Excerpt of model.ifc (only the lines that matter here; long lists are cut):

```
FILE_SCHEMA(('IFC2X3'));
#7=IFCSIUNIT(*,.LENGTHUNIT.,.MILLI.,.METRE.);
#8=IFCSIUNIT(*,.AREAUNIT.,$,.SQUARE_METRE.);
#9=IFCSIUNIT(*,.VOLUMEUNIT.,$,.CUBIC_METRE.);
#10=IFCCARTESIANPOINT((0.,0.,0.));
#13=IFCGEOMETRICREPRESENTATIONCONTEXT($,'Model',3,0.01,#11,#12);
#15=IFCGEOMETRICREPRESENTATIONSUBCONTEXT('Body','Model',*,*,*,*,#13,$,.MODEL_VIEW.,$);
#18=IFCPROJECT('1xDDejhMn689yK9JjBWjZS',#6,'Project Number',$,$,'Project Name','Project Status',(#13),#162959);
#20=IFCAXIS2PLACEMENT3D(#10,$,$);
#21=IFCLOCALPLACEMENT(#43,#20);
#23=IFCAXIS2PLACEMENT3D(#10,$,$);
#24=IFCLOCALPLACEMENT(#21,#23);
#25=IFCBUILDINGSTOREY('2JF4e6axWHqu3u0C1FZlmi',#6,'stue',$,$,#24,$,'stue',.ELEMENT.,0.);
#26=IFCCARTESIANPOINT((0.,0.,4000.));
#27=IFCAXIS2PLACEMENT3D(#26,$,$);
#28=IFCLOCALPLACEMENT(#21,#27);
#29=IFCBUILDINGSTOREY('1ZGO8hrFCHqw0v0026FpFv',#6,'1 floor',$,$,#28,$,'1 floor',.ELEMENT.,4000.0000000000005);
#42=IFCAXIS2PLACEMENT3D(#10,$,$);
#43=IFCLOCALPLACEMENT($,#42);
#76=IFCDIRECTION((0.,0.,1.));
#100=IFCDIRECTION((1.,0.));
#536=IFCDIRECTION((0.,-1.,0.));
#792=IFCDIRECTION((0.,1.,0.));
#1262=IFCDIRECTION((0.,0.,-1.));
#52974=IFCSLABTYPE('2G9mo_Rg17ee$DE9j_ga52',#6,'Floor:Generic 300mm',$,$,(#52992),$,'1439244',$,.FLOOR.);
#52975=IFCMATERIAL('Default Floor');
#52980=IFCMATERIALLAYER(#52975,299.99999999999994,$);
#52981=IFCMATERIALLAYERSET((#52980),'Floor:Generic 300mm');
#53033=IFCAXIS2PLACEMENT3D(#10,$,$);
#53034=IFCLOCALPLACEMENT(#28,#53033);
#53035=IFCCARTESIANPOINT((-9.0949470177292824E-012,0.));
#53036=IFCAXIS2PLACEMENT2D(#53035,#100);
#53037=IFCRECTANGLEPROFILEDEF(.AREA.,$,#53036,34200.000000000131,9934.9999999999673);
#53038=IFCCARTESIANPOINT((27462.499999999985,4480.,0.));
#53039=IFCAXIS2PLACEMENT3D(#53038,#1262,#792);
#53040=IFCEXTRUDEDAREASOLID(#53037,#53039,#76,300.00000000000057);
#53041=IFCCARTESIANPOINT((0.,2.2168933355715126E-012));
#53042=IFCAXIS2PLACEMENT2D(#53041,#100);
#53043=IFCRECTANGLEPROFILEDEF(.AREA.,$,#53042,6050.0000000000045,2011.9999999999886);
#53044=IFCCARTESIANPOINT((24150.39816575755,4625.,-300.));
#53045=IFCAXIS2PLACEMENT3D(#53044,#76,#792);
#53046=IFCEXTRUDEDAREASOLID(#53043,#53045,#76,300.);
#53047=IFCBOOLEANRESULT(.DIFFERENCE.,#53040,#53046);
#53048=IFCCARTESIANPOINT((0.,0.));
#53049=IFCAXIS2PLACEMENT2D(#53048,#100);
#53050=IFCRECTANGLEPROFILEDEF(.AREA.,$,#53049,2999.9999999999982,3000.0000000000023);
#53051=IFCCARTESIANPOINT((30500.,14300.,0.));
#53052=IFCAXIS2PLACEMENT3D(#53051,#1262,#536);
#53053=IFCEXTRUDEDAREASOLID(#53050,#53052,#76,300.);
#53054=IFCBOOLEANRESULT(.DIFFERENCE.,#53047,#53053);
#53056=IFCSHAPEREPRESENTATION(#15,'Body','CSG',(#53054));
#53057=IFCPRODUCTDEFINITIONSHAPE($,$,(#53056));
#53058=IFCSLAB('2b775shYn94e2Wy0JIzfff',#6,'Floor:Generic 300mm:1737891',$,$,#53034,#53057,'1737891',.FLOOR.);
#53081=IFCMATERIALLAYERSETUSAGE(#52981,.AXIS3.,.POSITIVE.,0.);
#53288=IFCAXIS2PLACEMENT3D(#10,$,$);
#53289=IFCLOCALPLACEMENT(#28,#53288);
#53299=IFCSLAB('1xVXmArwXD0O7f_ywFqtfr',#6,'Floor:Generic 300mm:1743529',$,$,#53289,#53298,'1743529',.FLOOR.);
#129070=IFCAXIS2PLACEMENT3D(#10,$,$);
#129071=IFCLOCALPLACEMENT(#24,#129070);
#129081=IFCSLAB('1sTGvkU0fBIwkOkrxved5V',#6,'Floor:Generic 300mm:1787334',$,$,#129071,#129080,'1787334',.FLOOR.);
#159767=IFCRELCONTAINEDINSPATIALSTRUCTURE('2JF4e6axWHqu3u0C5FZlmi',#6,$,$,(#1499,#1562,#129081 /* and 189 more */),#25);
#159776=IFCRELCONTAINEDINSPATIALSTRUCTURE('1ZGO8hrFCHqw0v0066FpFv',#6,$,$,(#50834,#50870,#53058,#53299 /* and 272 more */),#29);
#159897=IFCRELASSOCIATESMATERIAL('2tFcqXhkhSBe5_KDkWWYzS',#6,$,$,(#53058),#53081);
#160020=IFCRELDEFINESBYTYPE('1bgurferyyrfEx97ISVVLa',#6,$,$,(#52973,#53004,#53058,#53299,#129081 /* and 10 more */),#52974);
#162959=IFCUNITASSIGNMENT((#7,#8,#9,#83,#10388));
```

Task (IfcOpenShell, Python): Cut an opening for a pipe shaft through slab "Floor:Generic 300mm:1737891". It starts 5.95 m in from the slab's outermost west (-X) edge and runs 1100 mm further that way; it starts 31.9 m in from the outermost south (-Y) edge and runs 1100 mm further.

```python
import numpy as np
import ifcopenshell
import ifcopenshell.api.feature
import ifcopenshell.api.geometry
import ifcopenshell.api.root
import ifcopenshell.geom
import ifcopenshell.util.placement
import ifcopenshell.util.representation
import ifcopenshell.util.shape
import ifcopenshell.util.unit

model = ifcopenshell.open("model.ifc")
unit_scale = ifcopenshell.util.unit.calculate_unit_scale(model)
settings = ifcopenshell.geom.settings()


def volume(element):
    """Net volume in cubic metres, openings subtracted."""
    shape = ifcopenshell.geom.create_shape(settings, element)
    return ifcopenshell.util.shape.get_volume(shape.geometry)


slab = model.by_guid("2b775shYn94e2Wy0JIzfff")
before = volume(slab)

# Extent in the slab's own axes, in metres. The edges named are its -X and -Y sides.
slab_shape = ifcopenshell.geom.create_shape(settings, slab)
vertices = ifcopenshell.util.shape.get_vertices(slab_shape.geometry)
x_min, y_min, bottom = vertices.min(axis=0)
top = vertices[:, 2].max()

opening = ifcopenshell.api.root.create_entity(model, ifc_class="IfcOpeningElement", name="Pipe shaft opening")
context = ifcopenshell.util.representation.get_context(model, "Model", "Body", "MODEL_VIEW")
width, depth = 1.1, 1.1
outline = [(0.0, 0.0), (width, 0.0), (width, depth), (0.0, depth), (0.0, 0.0)]
# Overshoot both faces by 50 mm so the cut is clean.
shape = ifcopenshell.api.geometry.add_slab_representation(
    model, context=context, depth=top - bottom + 0.1, polyline=outline
)
ifcopenshell.api.geometry.assign_representation(model, product=opening, representation=shape)

matrix = ifcopenshell.util.placement.get_local_placement(slab.ObjectPlacement)
matrix[:, 3] = matrix @ np.append(np.array([x_min + 5.95, y_min + 31.9, bottom - 0.05]) / unit_scale, 1.0)
ifcopenshell.api.geometry.edit_object_placement(model, product=opening, matrix=matrix, is_si=False)
ifcopenshell.api.feature.add_feature(model, feature=opening, element=slab)

after = volume(slab)

print(f"slab volume {before:.3f} -> {after:.3f} m3")

model.write("model-out.ifc")
```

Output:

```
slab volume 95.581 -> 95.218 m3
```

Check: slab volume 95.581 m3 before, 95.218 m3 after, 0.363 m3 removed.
